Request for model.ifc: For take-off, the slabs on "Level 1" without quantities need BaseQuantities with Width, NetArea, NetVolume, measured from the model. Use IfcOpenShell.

First a look at what the model holds.

```python
import ifcopenshell
import ifcopenshell.util.element
import ifcopenshell.util.unit

model = ifcopenshell.open("model.ifc")
print(model.schema)
for unit_type in ("LENGTHUNIT", "AREAUNIT", "VOLUMEUNIT"):
    print(unit_type, ifcopenshell.util.unit.calculate_unit_scale(model, unit_type))
storey = next(s for s in model.by_type("IfcBuildingStorey") if s.Name == "Level 1")
slabs = [e for e in ifcopenshell.util.element.get_decomposition(storey) if e.is_a("IfcSlab")]
for e in sorted(slabs, key=lambda e: e.id()):
    print(e.id(), e.is_a(), e.Name, list(ifcopenshell.util.element.get_psets(e, qtos_only=True)), sep=" | ")
```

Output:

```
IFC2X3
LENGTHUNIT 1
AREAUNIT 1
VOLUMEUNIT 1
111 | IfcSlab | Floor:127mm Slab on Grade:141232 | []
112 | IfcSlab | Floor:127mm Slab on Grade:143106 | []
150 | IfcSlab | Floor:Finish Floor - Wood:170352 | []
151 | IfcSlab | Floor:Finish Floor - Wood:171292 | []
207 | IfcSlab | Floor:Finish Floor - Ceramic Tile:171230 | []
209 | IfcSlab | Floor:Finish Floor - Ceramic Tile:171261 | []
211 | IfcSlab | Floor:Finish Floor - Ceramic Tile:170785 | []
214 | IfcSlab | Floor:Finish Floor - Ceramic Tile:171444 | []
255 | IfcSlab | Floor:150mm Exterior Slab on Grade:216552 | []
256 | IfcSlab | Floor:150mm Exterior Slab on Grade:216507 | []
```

```python
import ifcopenshell
import ifcopenshell.api.pset
import ifcopenshell.geom
import ifcopenshell.util.element
import ifcopenshell.util.shape
import ifcopenshell.util.unit

model = ifcopenshell.open("model.ifc")
unit_scale = ifcopenshell.util.unit.calculate_unit_scale(model)
area_scale = ifcopenshell.util.unit.calculate_unit_scale(model, "AREAUNIT")
volume_scale = ifcopenshell.util.unit.calculate_unit_scale(model, "VOLUMEUNIT")
settings = ifcopenshell.geom.settings()

storey = next(s for s in model.by_type("IfcBuildingStorey") if s.Name == "Level 1")
slabs = [e for e in ifcopenshell.util.element.get_decomposition(storey) if e.is_a("IfcSlab")]

for e in sorted(slabs, key=lambda e: e.id()):
    if ifcopenshell.util.element.get_psets(e, qtos_only=True, should_inherit=False):
        continue
    # Geometry comes back in metres, in the element's own axes.
    shape = ifcopenshell.geom.create_shape(settings, e)
    values = {
        "Width": ifcopenshell.util.shape.get_z(shape.geometry) / unit_scale,
        "NetArea": ifcopenshell.util.shape.get_footprint_area(shape.geometry) / area_scale,
        "NetVolume": ifcopenshell.util.shape.get_volume(shape.geometry) / volume_scale,
    }
    qto = ifcopenshell.api.pset.add_qto(model, product=e, name="BaseQuantities")
    ifcopenshell.api.pset.edit_qto(model, qto=qto, properties=values)
    print(e.id(), {k: round(v, 3) for k, v in values.items()})

model.write("model_edited.ifc")
```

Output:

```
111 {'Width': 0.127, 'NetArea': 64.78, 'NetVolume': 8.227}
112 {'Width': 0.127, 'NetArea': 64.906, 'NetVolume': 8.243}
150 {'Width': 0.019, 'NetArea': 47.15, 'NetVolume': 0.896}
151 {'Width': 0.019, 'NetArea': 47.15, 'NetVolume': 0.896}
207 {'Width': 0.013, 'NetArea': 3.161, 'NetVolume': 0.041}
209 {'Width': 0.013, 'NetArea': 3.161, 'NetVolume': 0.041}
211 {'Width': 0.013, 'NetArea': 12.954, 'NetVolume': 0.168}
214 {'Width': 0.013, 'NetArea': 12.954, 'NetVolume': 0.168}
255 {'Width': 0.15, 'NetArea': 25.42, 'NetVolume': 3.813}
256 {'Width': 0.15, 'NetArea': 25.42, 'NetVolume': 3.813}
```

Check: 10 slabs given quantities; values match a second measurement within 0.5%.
